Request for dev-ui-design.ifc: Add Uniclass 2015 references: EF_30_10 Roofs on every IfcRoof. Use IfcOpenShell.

First a look at what the model holds.

```python
import ifcopenshell

model = ifcopenshell.open("dev-ui-design.ifc")
print(model.schema)
print("classifications:", [c.Name for c in model.by_type("IfcClassification")])
for ifc_class in ("IfcDoor", "IfcRoof", "IfcStair", "IfcWall", "IfcWindow"):
    print(ifc_class, len(model.by_type(ifc_class)))
```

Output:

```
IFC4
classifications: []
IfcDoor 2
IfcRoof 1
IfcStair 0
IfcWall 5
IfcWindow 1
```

```python
import ifcopenshell
import ifcopenshell.api.classification

model = ifcopenshell.open("dev-ui-design.ifc")

system = ifcopenshell.api.classification.add_classification(model, classification="Uniclass 2015")

codes = {
    "IfcRoof": ("EF_30_10", "Roofs"),
}
for ifc_class, (code, name) in codes.items():
    products = model.by_type(ifc_class)
    ifcopenshell.api.classification.add_reference(
        model, products=products, classification=system, identification=code, name=name
    )
    print(code, len(products))

model.write("dev-ui-design_edited.ifc")
```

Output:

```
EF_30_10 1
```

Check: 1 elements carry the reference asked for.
